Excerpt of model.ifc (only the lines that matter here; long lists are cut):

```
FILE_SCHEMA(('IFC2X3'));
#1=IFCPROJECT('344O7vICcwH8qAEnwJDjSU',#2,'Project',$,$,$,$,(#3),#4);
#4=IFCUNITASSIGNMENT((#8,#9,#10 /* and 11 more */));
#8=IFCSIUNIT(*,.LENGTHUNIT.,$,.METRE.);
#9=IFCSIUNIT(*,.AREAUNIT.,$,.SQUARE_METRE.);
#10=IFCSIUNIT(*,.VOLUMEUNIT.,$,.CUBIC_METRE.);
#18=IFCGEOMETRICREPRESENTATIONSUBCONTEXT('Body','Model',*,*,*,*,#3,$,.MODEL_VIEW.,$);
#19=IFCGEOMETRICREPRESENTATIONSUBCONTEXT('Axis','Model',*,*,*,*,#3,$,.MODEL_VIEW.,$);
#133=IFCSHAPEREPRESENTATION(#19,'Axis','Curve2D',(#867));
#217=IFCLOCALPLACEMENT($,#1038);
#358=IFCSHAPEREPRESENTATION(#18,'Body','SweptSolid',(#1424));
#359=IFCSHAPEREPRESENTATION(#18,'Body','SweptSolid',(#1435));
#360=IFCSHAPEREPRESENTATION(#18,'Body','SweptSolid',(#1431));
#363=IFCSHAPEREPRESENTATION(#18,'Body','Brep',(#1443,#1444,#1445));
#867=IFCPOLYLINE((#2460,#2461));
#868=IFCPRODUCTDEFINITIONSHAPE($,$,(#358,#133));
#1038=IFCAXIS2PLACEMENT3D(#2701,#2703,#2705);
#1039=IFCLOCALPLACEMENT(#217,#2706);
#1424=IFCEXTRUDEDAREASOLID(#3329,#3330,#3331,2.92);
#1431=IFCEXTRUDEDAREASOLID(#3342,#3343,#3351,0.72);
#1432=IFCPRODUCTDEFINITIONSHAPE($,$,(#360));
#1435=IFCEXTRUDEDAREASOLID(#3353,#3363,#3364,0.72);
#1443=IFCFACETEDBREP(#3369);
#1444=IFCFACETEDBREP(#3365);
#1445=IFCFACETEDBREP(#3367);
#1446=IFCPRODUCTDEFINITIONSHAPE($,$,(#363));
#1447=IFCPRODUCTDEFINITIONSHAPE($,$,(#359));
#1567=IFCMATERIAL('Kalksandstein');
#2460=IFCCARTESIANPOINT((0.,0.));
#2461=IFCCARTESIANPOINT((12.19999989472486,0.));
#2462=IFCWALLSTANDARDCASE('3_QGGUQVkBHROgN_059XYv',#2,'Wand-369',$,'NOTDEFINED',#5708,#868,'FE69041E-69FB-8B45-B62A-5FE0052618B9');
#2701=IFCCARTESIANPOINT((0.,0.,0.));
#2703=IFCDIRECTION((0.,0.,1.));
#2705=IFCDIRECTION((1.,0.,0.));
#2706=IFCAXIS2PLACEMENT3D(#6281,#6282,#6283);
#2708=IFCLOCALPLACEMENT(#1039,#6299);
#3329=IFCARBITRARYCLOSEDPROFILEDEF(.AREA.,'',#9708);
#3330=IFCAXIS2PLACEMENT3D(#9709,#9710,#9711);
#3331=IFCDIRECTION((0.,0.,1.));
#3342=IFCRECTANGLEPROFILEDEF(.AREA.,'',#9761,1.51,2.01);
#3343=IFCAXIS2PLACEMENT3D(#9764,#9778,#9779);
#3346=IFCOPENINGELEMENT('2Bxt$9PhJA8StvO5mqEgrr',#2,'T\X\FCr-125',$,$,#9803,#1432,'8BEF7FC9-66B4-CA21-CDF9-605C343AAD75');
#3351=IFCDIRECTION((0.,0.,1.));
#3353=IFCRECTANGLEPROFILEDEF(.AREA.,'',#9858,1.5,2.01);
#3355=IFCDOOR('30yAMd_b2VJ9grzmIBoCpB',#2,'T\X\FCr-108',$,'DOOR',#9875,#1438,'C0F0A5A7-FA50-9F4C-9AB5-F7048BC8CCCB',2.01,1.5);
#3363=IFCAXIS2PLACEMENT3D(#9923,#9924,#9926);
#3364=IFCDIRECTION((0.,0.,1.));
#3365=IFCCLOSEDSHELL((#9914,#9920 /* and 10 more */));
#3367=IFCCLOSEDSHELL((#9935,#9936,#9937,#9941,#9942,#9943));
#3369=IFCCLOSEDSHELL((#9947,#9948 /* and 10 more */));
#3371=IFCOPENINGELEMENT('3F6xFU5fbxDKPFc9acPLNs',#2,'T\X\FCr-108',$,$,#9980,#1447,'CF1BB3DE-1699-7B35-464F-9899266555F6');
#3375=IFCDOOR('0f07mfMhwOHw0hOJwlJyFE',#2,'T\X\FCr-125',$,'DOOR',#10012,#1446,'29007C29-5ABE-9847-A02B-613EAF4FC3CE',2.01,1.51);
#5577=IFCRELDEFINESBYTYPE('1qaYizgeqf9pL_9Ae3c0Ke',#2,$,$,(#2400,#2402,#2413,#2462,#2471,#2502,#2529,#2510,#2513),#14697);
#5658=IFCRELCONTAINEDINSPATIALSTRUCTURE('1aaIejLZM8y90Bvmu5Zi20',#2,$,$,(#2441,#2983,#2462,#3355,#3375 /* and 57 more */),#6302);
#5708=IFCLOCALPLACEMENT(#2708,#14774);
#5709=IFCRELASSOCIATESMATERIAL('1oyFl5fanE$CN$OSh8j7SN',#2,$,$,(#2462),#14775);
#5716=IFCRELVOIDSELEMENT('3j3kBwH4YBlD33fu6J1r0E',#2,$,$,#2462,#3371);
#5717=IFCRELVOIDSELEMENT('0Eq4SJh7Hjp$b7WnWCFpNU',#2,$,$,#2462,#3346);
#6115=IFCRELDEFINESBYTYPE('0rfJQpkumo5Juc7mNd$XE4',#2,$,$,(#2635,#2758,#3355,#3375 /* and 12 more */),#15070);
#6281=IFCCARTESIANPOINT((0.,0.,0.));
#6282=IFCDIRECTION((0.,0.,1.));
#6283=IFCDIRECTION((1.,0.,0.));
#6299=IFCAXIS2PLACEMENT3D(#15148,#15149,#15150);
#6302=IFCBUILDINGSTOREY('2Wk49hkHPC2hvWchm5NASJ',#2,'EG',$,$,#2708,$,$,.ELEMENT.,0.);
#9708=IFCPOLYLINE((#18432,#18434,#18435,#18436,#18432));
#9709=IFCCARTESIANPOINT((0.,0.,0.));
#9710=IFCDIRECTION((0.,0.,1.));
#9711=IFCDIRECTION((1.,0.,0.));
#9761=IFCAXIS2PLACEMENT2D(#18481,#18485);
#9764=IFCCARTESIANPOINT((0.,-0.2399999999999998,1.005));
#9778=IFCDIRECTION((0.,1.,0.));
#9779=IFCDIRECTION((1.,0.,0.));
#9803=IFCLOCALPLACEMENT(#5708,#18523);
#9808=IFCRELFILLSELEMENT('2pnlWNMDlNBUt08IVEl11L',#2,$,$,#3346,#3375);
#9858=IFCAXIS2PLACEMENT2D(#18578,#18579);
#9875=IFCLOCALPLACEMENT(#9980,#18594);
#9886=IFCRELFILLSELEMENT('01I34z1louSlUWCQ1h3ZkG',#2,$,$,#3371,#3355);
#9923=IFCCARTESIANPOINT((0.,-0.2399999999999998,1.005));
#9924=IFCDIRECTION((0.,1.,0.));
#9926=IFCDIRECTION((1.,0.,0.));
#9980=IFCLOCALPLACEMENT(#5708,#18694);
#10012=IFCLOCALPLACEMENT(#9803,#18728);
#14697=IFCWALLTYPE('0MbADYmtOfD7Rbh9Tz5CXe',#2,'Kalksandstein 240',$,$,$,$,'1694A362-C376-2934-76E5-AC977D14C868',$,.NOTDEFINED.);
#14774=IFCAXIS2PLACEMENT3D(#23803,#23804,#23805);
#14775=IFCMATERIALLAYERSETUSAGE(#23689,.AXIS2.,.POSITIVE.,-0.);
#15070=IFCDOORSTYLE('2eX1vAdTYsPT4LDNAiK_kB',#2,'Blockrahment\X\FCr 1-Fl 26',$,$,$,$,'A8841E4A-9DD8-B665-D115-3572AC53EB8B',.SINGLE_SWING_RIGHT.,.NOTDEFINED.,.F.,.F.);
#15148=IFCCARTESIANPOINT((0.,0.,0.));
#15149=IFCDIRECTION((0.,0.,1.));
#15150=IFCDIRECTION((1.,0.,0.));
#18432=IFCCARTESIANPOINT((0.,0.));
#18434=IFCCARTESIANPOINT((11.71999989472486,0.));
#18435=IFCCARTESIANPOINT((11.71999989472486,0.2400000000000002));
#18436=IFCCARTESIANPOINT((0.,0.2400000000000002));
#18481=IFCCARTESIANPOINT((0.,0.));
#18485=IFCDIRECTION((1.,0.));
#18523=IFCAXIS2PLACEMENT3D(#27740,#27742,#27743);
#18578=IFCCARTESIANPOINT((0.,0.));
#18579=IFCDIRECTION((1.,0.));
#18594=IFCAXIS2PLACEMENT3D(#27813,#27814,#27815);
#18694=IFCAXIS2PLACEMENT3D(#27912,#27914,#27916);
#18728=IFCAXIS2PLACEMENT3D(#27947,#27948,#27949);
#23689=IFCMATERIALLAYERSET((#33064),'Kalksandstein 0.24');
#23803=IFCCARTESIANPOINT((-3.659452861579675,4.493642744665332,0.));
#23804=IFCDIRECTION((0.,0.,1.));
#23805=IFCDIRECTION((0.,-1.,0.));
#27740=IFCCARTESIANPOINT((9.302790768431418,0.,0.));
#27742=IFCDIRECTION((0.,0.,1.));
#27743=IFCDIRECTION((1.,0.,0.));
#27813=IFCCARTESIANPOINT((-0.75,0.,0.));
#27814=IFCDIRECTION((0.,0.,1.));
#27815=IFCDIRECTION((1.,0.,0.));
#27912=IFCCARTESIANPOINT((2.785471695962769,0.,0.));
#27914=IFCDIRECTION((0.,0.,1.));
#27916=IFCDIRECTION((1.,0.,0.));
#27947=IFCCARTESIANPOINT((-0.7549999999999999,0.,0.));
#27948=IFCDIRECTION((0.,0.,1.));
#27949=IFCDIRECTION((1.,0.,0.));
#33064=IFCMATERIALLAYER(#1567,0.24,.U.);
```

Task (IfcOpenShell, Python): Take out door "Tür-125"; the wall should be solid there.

```python
import ifcopenshell
import ifcopenshell.api.feature
import ifcopenshell.api.root
import ifcopenshell.geom
import ifcopenshell.util.shape

model = ifcopenshell.open("model.ifc")
settings = ifcopenshell.geom.settings()


def volume(element):
    """Net volume in cubic metres, openings subtracted."""
    shape = ifcopenshell.geom.create_shape(settings, element)
    return ifcopenshell.util.shape.get_volume(shape.geometry)


door = model.by_guid("0f07mfMhwOHw0hOJwlJyFE")
opening = door.FillsVoids[0].RelatingOpeningElement
wall = opening.VoidsElements[0].RelatingBuildingElement
before = volume(wall)

ifcopenshell.api.root.remove_product(model, product=door)
ifcopenshell.api.feature.remove_feature(model, feature=opening)

after = volume(wall)

print(f"wall volume {before:.3f} -> {after:.3f} m3")

model.write("model_updated.ifc")
```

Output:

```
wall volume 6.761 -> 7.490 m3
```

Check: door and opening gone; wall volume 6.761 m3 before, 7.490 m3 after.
